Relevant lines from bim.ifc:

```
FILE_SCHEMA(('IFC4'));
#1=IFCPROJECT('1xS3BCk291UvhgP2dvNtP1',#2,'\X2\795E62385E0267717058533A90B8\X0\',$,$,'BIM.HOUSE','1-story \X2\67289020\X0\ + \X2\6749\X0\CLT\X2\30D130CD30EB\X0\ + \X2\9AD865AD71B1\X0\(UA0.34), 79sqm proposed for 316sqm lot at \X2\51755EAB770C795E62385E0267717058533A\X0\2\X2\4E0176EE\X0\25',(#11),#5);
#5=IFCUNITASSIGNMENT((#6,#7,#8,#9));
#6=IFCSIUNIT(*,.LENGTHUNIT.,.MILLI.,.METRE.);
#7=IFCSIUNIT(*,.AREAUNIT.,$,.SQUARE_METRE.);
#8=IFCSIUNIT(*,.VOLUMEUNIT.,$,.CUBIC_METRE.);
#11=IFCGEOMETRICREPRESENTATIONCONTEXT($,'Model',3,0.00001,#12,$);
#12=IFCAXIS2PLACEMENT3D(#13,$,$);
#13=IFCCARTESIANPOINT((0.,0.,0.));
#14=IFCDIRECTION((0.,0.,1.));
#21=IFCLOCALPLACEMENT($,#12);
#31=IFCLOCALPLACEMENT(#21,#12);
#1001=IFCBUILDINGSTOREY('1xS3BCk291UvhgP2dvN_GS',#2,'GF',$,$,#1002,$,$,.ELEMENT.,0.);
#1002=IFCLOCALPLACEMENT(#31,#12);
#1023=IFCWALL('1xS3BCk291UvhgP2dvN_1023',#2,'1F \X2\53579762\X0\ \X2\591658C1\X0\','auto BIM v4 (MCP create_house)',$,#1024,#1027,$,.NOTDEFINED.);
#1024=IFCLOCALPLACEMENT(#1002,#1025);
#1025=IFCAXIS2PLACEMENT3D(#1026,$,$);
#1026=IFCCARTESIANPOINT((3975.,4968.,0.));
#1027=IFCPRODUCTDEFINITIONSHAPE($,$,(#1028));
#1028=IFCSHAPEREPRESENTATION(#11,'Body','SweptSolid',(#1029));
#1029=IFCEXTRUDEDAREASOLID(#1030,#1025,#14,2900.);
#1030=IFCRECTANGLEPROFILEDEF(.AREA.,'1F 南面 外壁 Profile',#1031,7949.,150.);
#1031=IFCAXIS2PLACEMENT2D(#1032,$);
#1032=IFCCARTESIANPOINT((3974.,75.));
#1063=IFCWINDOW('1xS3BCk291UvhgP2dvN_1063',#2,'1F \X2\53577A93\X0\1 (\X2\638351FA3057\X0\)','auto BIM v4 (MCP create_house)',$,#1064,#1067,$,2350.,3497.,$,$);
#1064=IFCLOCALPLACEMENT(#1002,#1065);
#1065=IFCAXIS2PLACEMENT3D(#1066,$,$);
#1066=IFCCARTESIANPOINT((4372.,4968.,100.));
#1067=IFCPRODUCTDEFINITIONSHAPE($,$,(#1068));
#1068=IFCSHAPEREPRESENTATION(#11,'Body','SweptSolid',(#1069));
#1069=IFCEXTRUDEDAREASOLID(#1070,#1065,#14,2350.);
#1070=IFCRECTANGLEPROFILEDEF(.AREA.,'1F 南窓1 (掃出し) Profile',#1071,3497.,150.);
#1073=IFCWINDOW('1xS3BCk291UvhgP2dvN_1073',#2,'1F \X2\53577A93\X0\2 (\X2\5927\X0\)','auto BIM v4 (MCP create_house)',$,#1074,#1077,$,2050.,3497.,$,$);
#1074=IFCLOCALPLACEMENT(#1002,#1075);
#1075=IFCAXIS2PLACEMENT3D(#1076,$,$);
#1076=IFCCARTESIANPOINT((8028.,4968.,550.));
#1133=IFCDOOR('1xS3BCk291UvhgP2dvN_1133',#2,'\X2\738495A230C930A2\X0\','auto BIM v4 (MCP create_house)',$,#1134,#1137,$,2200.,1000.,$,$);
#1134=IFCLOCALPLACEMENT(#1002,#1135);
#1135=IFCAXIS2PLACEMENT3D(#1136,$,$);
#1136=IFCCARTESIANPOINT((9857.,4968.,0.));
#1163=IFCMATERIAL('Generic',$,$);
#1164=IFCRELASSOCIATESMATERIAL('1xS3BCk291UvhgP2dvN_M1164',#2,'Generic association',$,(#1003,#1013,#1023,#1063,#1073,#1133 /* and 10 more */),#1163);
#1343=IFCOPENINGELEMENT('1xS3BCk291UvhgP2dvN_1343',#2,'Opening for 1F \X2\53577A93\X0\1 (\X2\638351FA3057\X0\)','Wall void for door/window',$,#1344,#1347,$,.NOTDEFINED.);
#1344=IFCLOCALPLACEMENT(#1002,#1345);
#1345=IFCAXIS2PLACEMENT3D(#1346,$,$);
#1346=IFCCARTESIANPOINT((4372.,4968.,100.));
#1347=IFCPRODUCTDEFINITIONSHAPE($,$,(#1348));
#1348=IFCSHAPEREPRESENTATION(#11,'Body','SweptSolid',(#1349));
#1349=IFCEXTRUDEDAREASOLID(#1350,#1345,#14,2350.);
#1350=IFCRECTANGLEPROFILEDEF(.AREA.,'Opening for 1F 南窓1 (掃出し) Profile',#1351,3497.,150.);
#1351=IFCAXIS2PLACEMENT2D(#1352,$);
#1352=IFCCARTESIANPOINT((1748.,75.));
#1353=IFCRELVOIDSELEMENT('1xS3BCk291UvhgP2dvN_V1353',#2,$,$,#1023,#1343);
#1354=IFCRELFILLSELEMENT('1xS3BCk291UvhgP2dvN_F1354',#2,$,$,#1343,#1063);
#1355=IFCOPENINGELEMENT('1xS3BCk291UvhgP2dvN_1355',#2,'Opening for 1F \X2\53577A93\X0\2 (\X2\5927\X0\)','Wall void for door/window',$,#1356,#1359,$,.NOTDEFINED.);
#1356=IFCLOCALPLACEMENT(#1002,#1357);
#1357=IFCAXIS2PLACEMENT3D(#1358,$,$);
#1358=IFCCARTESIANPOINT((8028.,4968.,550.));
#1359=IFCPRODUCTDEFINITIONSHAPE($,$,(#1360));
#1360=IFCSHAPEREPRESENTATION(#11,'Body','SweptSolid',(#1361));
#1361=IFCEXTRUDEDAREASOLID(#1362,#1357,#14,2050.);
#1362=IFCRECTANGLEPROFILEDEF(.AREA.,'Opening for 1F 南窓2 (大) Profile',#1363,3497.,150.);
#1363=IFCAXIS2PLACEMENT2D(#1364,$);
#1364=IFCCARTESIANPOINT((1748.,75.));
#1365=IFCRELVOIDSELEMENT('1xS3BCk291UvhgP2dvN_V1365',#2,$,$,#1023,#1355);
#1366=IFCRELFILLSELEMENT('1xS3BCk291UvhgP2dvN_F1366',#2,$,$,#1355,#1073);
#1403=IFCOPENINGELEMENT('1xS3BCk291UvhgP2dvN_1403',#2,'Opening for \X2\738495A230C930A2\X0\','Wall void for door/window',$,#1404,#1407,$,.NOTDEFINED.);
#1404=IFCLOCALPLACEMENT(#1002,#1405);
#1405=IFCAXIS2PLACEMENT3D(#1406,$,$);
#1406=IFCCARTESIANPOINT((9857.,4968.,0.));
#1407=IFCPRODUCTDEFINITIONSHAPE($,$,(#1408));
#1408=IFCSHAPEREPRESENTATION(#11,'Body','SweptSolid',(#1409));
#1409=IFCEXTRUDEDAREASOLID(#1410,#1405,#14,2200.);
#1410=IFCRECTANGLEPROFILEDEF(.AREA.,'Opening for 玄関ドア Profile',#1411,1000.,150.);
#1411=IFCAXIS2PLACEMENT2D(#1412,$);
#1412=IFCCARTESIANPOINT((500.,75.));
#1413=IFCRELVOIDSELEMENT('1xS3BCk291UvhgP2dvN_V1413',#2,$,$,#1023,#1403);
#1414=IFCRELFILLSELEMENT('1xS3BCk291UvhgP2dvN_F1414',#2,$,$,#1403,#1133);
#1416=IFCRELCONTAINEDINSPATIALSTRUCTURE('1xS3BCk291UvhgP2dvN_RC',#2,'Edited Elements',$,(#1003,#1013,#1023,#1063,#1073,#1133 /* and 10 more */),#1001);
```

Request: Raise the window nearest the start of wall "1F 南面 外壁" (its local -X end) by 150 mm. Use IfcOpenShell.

```python
import numpy as np
import ifcopenshell
import ifcopenshell.api.geometry
import ifcopenshell.util.placement
import ifcopenshell.util.unit

model = ifcopenshell.open("bim.ifc")
unit_scale = ifcopenshell.util.unit.calculate_unit_scale(model)

window = model.by_guid("1xS3BCk291UvhgP2dvN_1063")
opening = window.FillsVoids[0].RelatingOpeningElement
dz = 0.15 / unit_scale

shift = np.array([0.0, 0.0, dz])
# The window is not placed relative to its opening, so move both.
for product in (opening, window):
    matrix = ifcopenshell.util.placement.get_local_placement(product.ObjectPlacement)
    matrix[:3, 3] += shift
    ifcopenshell.api.geometry.edit_object_placement(model, product=product, matrix=matrix, is_si=False)

print(f"moved by {dz * unit_scale:+.3f} m")

model.write("bim_v2.ifc")
```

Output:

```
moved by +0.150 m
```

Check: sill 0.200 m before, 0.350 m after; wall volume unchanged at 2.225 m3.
